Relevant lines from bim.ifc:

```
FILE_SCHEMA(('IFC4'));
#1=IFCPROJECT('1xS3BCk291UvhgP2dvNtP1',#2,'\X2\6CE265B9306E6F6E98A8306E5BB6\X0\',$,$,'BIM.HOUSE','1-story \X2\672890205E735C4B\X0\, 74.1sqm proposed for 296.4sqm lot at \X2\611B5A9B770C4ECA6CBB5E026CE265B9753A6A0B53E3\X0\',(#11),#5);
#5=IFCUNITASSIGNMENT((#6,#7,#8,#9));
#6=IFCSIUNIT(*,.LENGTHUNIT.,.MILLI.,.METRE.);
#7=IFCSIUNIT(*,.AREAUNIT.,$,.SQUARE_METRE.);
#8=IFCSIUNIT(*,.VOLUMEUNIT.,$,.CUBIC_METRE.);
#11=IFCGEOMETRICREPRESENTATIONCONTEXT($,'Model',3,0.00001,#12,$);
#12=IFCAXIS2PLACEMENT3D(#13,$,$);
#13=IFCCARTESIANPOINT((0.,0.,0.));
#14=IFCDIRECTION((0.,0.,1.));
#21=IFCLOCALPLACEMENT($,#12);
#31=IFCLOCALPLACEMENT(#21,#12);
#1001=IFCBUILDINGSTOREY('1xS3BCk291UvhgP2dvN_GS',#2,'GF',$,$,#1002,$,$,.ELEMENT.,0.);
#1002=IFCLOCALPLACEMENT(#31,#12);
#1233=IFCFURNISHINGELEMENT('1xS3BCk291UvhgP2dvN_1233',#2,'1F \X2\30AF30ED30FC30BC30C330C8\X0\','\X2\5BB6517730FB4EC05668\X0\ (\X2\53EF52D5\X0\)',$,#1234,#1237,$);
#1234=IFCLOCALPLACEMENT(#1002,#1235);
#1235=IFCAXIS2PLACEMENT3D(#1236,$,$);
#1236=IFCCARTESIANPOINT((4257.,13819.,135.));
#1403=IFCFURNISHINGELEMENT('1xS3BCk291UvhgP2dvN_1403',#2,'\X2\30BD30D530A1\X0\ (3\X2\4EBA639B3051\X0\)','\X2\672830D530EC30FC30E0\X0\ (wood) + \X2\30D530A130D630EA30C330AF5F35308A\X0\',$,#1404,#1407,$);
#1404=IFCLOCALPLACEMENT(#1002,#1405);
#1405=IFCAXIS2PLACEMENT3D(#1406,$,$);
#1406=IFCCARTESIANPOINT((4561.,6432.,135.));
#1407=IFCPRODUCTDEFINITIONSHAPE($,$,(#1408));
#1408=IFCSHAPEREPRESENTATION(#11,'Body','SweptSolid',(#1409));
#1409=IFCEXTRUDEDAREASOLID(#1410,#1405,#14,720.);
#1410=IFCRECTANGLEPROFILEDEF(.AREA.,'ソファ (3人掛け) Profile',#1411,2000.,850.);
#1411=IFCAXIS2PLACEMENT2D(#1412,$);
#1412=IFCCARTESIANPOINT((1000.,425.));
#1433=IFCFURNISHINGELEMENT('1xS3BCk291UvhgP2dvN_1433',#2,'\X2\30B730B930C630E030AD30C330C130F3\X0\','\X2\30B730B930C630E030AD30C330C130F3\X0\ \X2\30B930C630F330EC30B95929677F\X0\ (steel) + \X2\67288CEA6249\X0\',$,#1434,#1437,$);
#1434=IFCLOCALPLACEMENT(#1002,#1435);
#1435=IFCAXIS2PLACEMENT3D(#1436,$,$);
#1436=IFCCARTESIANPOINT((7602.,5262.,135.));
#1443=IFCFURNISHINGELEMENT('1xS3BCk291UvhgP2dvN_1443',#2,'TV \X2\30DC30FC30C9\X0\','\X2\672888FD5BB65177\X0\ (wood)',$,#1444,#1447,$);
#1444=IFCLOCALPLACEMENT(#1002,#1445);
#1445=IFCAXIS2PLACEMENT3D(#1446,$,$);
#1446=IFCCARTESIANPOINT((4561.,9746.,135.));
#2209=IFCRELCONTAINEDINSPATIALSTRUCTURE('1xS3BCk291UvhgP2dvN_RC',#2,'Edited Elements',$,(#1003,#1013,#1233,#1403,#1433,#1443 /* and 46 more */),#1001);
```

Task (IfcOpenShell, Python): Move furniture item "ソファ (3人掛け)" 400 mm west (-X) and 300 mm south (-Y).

```python
import ifcopenshell
import ifcopenshell.api.geometry
import ifcopenshell.util.placement
import ifcopenshell.util.unit

model = ifcopenshell.open("bim.ifc")
unit_scale = ifcopenshell.util.unit.calculate_unit_scale(model)

item = model.by_guid("1xS3BCk291UvhgP2dvN_1403")
matrix = ifcopenshell.util.placement.get_local_placement(item.ObjectPlacement)
matrix[0, 3] -= 0.4 / unit_scale
matrix[1, 3] -= 0.3 / unit_scale
ifcopenshell.api.geometry.edit_object_placement(model, product=item, matrix=matrix, is_si=False)

print(ifcopenshell.util.placement.get_local_placement(item.ObjectPlacement).round(3) + 0.0)

model.write("bim_v2.ifc")
```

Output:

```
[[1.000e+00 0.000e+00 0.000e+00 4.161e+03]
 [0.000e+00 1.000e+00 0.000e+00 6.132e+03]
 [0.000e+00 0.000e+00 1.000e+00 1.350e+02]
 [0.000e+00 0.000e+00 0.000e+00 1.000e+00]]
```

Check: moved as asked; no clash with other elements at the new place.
